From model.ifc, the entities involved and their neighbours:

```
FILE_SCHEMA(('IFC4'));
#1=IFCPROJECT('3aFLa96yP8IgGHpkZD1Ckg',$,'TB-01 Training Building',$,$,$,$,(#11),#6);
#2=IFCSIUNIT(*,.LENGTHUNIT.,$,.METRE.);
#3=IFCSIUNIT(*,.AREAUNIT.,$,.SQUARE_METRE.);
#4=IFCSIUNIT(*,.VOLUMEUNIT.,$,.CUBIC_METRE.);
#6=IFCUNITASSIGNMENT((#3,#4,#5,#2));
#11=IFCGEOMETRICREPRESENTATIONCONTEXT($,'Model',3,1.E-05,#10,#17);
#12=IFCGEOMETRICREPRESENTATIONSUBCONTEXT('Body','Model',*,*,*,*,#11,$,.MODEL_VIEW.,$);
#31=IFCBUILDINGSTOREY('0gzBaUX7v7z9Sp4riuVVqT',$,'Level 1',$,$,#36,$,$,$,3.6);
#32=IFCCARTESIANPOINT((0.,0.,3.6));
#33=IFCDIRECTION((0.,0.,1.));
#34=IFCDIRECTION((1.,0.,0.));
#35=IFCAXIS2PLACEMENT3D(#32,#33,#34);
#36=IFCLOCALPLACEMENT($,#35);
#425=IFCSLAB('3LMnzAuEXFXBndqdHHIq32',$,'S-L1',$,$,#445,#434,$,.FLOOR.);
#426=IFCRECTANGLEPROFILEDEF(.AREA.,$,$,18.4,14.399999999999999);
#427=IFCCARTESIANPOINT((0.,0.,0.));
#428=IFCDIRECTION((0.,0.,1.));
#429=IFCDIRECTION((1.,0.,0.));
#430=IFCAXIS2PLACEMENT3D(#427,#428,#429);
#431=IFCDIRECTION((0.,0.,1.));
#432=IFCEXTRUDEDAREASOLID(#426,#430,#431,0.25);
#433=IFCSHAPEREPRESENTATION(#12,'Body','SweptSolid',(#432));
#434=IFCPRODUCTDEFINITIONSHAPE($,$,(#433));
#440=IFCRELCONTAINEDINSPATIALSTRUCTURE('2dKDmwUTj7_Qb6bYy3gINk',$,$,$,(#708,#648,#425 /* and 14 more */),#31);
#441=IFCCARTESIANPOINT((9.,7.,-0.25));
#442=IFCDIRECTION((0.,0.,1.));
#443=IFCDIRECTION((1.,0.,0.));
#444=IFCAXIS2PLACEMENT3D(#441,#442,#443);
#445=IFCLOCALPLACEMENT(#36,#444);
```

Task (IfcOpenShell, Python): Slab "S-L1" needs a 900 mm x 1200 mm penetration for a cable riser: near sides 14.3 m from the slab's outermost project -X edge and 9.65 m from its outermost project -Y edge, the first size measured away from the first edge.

```python
import numpy as np
import ifcopenshell
import ifcopenshell.api.feature
import ifcopenshell.api.geometry
import ifcopenshell.api.root
import ifcopenshell.geom
import ifcopenshell.util.placement
import ifcopenshell.util.representation
import ifcopenshell.util.shape
import ifcopenshell.util.unit

model = ifcopenshell.open("model.ifc")
unit_scale = ifcopenshell.util.unit.calculate_unit_scale(model)
settings = ifcopenshell.geom.settings()


def volume(element):
    """Net volume in cubic metres, openings subtracted."""
    shape = ifcopenshell.geom.create_shape(settings, element)
    return ifcopenshell.util.shape.get_volume(shape.geometry)


slab = model.by_guid("3LMnzAuEXFXBndqdHHIq32")
before = volume(slab)

# Extent in the slab's own axes, in metres. The edges named are its -X and -Y sides.
slab_shape = ifcopenshell.geom.create_shape(settings, slab)
vertices = ifcopenshell.util.shape.get_vertices(slab_shape.geometry)
x_min, y_min, bottom = vertices.min(axis=0)
top = vertices[:, 2].max()

opening = ifcopenshell.api.root.create_entity(model, ifc_class="IfcOpeningElement", name="Cable riser opening", predefined_type="OPENING")
context = ifcopenshell.util.representation.get_context(model, "Model", "Body", "MODEL_VIEW")
width, depth = 0.9, 1.2
outline = [(0.0, 0.0), (width, 0.0), (width, depth), (0.0, depth), (0.0, 0.0)]
# Overshoot both faces by 50 mm so the cut is clean.
shape = ifcopenshell.api.geometry.add_slab_representation(
    model, context=context, depth=top - bottom + 0.1, polyline=outline
)
ifcopenshell.api.geometry.assign_representation(model, product=opening, representation=shape)

matrix = ifcopenshell.util.placement.get_local_placement(slab.ObjectPlacement)
matrix[:, 3] = matrix @ np.append(np.array([x_min + 14.3, y_min + 9.65, bottom - 0.05]) / unit_scale, 1.0)
ifcopenshell.api.geometry.edit_object_placement(model, product=opening, matrix=matrix, is_si=False)
ifcopenshell.api.feature.add_feature(model, feature=opening, element=slab)

after = volume(slab)

print(f"slab volume {before:.3f} -> {after:.3f} m3")

model.write("model_rev.ifc")
```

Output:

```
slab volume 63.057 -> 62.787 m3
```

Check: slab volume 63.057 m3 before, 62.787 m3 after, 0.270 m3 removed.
